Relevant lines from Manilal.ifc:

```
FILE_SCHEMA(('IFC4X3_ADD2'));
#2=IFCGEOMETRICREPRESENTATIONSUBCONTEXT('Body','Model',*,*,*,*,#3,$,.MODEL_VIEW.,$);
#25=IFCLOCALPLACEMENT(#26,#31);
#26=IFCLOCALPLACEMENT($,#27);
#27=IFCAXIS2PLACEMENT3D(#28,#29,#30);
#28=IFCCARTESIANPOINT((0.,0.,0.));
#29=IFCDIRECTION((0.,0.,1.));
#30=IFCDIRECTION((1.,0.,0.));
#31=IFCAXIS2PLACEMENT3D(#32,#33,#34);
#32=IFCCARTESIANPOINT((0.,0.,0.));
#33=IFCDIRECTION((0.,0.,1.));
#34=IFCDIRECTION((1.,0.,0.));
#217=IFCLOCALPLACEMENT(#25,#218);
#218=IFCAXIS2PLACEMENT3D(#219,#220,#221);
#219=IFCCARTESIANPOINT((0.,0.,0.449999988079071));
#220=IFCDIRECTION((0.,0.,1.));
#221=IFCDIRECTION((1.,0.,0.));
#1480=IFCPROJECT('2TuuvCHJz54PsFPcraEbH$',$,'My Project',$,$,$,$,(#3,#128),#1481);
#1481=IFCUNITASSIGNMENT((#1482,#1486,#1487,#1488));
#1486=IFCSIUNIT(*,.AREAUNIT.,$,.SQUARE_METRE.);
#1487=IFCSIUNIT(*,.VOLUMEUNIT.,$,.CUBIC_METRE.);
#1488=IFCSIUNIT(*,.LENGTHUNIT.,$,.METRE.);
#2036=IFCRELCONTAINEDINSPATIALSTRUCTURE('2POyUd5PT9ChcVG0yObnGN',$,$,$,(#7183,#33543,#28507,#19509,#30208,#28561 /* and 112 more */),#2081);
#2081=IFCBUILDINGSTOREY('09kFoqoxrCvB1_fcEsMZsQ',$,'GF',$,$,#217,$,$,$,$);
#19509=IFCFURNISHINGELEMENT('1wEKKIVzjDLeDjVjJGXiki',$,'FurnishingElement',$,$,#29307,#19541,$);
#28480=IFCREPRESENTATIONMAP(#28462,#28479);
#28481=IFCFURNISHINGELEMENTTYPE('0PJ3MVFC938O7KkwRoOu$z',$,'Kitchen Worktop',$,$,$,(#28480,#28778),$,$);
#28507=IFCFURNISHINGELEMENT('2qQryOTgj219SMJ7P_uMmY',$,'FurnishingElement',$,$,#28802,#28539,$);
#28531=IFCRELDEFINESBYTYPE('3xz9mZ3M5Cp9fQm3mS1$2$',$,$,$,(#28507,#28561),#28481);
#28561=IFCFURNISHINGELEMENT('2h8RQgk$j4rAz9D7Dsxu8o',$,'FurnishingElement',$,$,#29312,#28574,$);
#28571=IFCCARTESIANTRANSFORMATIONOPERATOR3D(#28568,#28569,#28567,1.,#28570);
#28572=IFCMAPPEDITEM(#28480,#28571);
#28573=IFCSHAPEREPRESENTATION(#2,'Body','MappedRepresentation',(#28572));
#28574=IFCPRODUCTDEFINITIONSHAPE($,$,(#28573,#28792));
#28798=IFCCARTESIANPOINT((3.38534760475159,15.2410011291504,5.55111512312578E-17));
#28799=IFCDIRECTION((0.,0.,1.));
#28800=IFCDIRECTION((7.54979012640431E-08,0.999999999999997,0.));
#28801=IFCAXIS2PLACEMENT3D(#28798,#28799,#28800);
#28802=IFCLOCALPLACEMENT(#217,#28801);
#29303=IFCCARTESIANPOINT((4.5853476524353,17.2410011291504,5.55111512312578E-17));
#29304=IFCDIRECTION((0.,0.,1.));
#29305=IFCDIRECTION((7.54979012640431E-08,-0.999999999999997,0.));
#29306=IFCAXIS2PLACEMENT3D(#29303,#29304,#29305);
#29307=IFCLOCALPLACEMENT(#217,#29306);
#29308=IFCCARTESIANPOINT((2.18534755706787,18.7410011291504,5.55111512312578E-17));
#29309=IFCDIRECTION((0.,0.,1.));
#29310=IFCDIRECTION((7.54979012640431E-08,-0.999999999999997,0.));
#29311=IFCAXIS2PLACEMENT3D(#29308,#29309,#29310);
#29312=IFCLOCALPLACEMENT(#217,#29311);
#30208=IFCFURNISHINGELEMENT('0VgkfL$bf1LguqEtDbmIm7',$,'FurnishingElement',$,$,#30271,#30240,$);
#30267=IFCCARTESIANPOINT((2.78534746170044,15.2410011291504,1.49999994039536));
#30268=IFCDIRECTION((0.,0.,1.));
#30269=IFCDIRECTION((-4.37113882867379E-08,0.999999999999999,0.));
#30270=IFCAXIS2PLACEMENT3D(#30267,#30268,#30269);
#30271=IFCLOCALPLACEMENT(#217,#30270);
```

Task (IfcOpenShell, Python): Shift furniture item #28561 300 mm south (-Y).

```python
import ifcopenshell
import ifcopenshell.api.geometry
import ifcopenshell.util.placement

model = ifcopenshell.open("Manilal.ifc")

item = model.by_guid("2h8RQgk$j4rAz9D7Dsxu8o")
matrix = ifcopenshell.util.placement.get_local_placement(item.ObjectPlacement)
matrix[1, 3] -= 0.3
ifcopenshell.api.geometry.edit_object_placement(model, product=item, matrix=matrix, is_si=False)

print(ifcopenshell.util.placement.get_local_placement(item.ObjectPlacement).round(3) + 0.0)

model.write("Manilal_updated.ifc")
```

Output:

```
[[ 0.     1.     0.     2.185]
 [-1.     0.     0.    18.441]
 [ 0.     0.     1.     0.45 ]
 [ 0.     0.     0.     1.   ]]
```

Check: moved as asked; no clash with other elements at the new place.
